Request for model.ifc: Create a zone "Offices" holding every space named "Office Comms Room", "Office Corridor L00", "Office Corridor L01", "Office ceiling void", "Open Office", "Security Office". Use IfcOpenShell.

First a look at what the model holds.

```python
import ifcopenshell

model = ifcopenshell.open("model.ifc")
print(model.schema)
seen = {}
for space in model.by_type("IfcSpace"):
    seen[space.LongName] = seen.get(space.LongName, 0) + 1
for name, count in sorted(seen.items(), key=str):
    print(count, "x", name)
print("zones:", [z.Name for z in model.by_type("IfcZone")][:20])
```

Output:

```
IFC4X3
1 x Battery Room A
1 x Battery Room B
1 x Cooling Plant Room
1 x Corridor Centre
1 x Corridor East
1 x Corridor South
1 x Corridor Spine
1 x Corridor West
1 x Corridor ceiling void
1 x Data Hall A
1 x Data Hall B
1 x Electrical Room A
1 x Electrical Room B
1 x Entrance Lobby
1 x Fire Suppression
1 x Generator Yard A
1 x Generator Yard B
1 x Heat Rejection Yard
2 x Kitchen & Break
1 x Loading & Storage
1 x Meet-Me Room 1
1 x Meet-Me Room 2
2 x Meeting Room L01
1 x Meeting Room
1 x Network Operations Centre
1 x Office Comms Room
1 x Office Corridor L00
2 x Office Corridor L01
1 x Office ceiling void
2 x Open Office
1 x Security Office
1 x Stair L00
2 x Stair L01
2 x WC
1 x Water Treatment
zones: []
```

```python
import ifcopenshell
import ifcopenshell.api.group
import ifcopenshell.api.root

model = ifcopenshell.open("model.ifc")

names = {"Office Comms Room", "Office Corridor L00", "Office Corridor L01", "Office ceiling void", "Open Office", "Security Office"}
spaces = [s for s in model.by_type("IfcSpace") if s.LongName in names]

zone = ifcopenshell.api.root.create_entity(model, ifc_class="IfcZone", name="Offices")
ifcopenshell.api.group.assign_group(model, products=spaces, group=zone)
print(len(spaces), "spaces in", zone.Name)

model.write("model_edited.ifc")
```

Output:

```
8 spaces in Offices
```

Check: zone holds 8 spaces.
